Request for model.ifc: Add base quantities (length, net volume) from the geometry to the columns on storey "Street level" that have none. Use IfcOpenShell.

First a look at what the model holds.

```python
import ifcopenshell
import ifcopenshell.util.element
import ifcopenshell.util.unit

model = ifcopenshell.open("model.ifc")
print(model.schema)
for unit_type in ("LENGTHUNIT", "AREAUNIT", "VOLUMEUNIT"):
    print(unit_type, ifcopenshell.util.unit.calculate_unit_scale(model, unit_type))
storey = next(s for s in model.by_type("IfcBuildingStorey") if s.Name == "Street level")
columns = [e for e in ifcopenshell.util.element.get_decomposition(storey) if e.is_a("IfcColumn")]
for e in sorted(columns, key=lambda e: e.id()):
    print(e.id(), e.is_a(), e.Name, list(ifcopenshell.util.element.get_psets(e, qtos_only=True)), sep=" | ")
```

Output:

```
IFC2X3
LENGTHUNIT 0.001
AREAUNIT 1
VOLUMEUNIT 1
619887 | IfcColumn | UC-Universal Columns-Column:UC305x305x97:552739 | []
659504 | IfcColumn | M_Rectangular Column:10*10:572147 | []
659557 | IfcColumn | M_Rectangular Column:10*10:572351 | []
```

```python
import ifcopenshell
import ifcopenshell.api.pset
import ifcopenshell.geom
import ifcopenshell.util.element
import ifcopenshell.util.shape
import ifcopenshell.util.unit

model = ifcopenshell.open("model.ifc")
unit_scale = ifcopenshell.util.unit.calculate_unit_scale(model)
volume_scale = ifcopenshell.util.unit.calculate_unit_scale(model, "VOLUMEUNIT")
settings = ifcopenshell.geom.settings()

storey = next(s for s in model.by_type("IfcBuildingStorey") if s.Name == "Street level")
columns = [e for e in ifcopenshell.util.element.get_decomposition(storey) if e.is_a("IfcColumn")]

for e in sorted(columns, key=lambda e: e.id()):
    if ifcopenshell.util.element.get_psets(e, qtos_only=True, should_inherit=False):
        continue
    # Geometry comes back in metres, in the element's own axes.
    shape = ifcopenshell.geom.create_shape(settings, e)
    values = {
        "Length": ifcopenshell.util.shape.get_z(shape.geometry) / unit_scale,
        "NetVolume": ifcopenshell.util.shape.get_volume(shape.geometry) / volume_scale,
    }
    qto = ifcopenshell.api.pset.add_qto(model, product=e, name="BaseQuantities")
    ifcopenshell.api.pset.edit_qto(model, qto=qto, properties=values)
    print(e.id(), {k: round(v, 3) for k, v in values.items()})

model.write("model-out.ifc")
```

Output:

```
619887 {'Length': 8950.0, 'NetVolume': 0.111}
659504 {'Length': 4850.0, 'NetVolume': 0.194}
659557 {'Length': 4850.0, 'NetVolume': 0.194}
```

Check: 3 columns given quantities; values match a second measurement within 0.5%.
